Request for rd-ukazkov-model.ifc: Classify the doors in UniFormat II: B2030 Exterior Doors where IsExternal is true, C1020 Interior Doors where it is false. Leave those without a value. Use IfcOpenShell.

First a look at what the model holds.

```python
import ifcopenshell
import ifcopenshell.util.element

model = ifcopenshell.open("rd-ukazkov-model.ifc")
print(model.schema)
print("classifications:", [c.Name for c in model.by_type("IfcClassification")])
values = [ifcopenshell.util.element.get_pset(e, "Pset_DoorCommon", "IsExternal") for e in model.by_type("IfcDoor")]
for value in (True, False, None):
    print("IsExternal", value, values.count(value))
```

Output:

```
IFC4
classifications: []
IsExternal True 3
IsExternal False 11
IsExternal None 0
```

```python
import ifcopenshell
import ifcopenshell.api.classification
import ifcopenshell.util.element

model = ifcopenshell.open("rd-ukazkov-model.ifc")

system = ifcopenshell.api.classification.add_classification(model, classification="UniFormat II")

doors = model.by_type("IfcDoor")
external = {e: ifcopenshell.util.element.get_pset(e, "Pset_DoorCommon", "IsExternal") for e in doors}
for flag, code, name in ((True, "B2030", "Exterior Doors"), (False, "C1020", "Interior Doors")):
    products = [e for e in doors if external[e] is flag]
    ifcopenshell.api.classification.add_reference(
        model, products=products, classification=system, identification=code, name=name
    )
    print(code, len(products))

model.write("rd-ukazkov-model_v2.ifc")
```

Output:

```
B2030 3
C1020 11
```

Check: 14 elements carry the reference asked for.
